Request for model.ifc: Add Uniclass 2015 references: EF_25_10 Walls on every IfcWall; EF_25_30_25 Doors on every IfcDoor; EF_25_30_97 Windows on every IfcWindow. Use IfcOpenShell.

First a look at what the model holds.

```python
import ifcopenshell

model = ifcopenshell.open("model.ifc")
print(model.schema)
print("classifications:", [c.Name for c in model.by_type("IfcClassification")])
for ifc_class in ("IfcDoor", "IfcRoof", "IfcStair", "IfcWall", "IfcWindow"):
    print(ifc_class, len(model.by_type(ifc_class)))
```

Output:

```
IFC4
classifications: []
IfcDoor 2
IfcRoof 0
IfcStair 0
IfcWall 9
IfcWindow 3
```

```python
import ifcopenshell
import ifcopenshell.api.classification

model = ifcopenshell.open("model.ifc")

system = ifcopenshell.api.classification.add_classification(model, classification="Uniclass 2015")

codes = {
    "IfcWall": ("EF_25_10", "Walls"),
    "IfcDoor": ("EF_25_30_25", "Doors"),
    "IfcWindow": ("EF_25_30_97", "Windows"),
}
for ifc_class, (code, name) in codes.items():
    products = model.by_type(ifc_class)
    ifcopenshell.api.classification.add_reference(
        model, products=products, classification=system, identification=code, name=name
    )
    print(code, len(products))

model.write("model_edited.ifc")
```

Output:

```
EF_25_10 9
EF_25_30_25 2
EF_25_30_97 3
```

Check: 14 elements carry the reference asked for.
